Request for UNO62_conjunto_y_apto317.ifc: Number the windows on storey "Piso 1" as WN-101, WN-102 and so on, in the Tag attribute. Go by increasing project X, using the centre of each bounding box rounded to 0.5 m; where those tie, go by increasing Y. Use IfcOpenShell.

First a look at what the model holds.

```python
import ifcopenshell
import ifcopenshell.util.element
import ifcopenshell.util.placement

model = ifcopenshell.open("UNO62_conjunto_y_apto317.ifc")
print(model.schema)
storey = next(s for s in model.by_type("IfcBuildingStorey") if s.Name == "Piso 1")
windows = [e for e in ifcopenshell.util.element.get_decomposition(storey) if e.is_a("IfcWindow")]
for e in sorted(windows, key=lambda e: e.id()):
    origin = ifcopenshell.util.placement.get_local_placement(e.ObjectPlacement)[:3, 3]
    print(e.id(), e.Tag, e.Name, origin.round(2) + 0.0, sep=" | ")
```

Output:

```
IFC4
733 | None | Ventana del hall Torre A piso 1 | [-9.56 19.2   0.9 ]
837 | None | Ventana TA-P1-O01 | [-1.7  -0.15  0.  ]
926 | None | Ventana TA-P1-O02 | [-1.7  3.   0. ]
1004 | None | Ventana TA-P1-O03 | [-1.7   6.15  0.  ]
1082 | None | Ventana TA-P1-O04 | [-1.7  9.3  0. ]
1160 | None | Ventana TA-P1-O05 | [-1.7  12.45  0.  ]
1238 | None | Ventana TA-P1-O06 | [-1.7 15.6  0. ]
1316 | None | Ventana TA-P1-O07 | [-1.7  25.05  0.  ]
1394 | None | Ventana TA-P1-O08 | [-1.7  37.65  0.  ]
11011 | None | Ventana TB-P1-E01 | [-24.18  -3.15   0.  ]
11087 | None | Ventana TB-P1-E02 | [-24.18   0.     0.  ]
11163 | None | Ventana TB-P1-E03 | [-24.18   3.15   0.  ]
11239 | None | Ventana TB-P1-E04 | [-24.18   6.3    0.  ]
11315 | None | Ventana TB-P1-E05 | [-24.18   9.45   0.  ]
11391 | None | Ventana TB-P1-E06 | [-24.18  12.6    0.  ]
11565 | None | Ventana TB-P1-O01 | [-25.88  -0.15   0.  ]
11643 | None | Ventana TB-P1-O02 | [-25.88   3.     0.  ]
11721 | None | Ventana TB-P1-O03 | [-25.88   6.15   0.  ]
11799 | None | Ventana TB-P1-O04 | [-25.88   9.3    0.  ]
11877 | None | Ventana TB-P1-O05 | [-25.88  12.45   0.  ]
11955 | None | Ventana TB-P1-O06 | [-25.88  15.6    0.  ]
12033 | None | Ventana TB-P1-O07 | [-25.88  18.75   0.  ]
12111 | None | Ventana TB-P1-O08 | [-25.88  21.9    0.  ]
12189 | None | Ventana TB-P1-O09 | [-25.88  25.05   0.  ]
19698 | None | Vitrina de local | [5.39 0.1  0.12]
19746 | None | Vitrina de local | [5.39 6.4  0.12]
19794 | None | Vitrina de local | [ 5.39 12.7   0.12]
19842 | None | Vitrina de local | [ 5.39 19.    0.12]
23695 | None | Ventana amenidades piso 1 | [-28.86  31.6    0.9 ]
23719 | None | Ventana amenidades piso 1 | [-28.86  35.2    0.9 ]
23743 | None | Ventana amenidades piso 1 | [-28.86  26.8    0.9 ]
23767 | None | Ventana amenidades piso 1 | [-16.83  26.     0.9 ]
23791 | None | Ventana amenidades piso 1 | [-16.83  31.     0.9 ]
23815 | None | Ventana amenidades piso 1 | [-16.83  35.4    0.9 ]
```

```python
import ifcopenshell
import ifcopenshell.geom
import ifcopenshell.util.element
import ifcopenshell.util.shape

model = ifcopenshell.open("UNO62_conjunto_y_apto317.ifc")
settings = ifcopenshell.geom.settings()
settings.set("use-world-coords", True)


def centre(element):
    shape = ifcopenshell.geom.create_shape(settings, element)
    return ifcopenshell.util.shape.get_bbox_centroid(shape.geometry)


storey = next(s for s in model.by_type("IfcBuildingStorey") if s.Name == "Piso 1")
windows = [e for e in ifcopenshell.util.element.get_decomposition(storey) if e.is_a("IfcWindow")]

# Insertion points can sit at a corner or the storey origin, so sort by the geometry (in metres).
centres = {e: centre(e) for e in windows}
windows.sort(key=lambda e: (round(centres[e][0] / 0.5), centres[e][1]))

for i, e in enumerate(windows, start=1):
    number = f"WN-1{i:02d}"
    e.Tag = number
    print(e.id(), number)

model.write("UNO62_conjunto_y_apto317_rev.ifc")
```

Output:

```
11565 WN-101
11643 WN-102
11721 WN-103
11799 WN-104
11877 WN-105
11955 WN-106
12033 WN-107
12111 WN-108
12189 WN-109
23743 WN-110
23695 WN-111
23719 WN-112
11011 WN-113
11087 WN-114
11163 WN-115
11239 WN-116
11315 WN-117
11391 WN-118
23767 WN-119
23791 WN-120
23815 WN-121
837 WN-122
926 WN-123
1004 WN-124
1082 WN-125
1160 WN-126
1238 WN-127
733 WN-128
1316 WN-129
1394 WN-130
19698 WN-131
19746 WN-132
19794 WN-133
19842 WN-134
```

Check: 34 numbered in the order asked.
